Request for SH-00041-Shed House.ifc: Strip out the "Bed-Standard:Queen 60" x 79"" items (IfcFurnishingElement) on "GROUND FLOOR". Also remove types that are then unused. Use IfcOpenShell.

First a look at what the model holds.

```python
import ifcopenshell
import ifcopenshell.util.element

model = ifcopenshell.open("SH-00041-Shed House.ifc")
print(model.schema)
storey = next(s for s in model.by_type("IfcBuildingStorey") if s.Name == "GROUND FLOOR")
furniture = [e for e in ifcopenshell.util.element.get_decomposition(storey) if e.is_a("IfcFurnishingElement")]
seen = {}
for e in furniture:
    element_type = ifcopenshell.util.element.get_type(e)
    name = element_type.Name if element_type not in (None, e) else None
    seen[name] = seen.get(name, 0) + 1
for name, count in sorted(seen.items(), key=str):
    print(count, "x", name)
```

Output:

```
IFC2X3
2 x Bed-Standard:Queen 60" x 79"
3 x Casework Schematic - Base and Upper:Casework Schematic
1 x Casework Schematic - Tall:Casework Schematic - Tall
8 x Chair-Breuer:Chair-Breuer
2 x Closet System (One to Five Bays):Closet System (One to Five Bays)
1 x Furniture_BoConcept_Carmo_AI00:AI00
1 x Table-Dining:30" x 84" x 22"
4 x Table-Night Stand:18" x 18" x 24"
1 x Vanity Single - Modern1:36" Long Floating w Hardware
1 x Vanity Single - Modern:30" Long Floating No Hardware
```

```python
import ifcopenshell
import ifcopenshell.api.root
import ifcopenshell.util.element

model = ifcopenshell.open("SH-00041-Shed House.ifc")

storey = next(s for s in model.by_type("IfcBuildingStorey") if s.Name == "GROUND FLOOR")
furniture = [e for e in ifcopenshell.util.element.get_decomposition(storey) if e.is_a("IfcFurnishingElement")]
targets = [e for e in furniture if (t := ifcopenshell.util.element.get_type(e)) not in (None, e) and t.Name == 'Bed-Standard:Queen 60" x 79"']
types = {ifcopenshell.util.element.get_type(e) for e in targets} - {None, *targets}

for e in targets:
    ifcopenshell.api.root.remove_product(model, product=e)
print(len(targets), "removed")

unused = [t for t in types if not ifcopenshell.util.element.get_types(t)]
for t in unused:
    ifcopenshell.api.root.remove_product(model, product=t)
print(len(unused), "unused types removed")

model.write("SH-00041-Shed House_rev.ifc")
```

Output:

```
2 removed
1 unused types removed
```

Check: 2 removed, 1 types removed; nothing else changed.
